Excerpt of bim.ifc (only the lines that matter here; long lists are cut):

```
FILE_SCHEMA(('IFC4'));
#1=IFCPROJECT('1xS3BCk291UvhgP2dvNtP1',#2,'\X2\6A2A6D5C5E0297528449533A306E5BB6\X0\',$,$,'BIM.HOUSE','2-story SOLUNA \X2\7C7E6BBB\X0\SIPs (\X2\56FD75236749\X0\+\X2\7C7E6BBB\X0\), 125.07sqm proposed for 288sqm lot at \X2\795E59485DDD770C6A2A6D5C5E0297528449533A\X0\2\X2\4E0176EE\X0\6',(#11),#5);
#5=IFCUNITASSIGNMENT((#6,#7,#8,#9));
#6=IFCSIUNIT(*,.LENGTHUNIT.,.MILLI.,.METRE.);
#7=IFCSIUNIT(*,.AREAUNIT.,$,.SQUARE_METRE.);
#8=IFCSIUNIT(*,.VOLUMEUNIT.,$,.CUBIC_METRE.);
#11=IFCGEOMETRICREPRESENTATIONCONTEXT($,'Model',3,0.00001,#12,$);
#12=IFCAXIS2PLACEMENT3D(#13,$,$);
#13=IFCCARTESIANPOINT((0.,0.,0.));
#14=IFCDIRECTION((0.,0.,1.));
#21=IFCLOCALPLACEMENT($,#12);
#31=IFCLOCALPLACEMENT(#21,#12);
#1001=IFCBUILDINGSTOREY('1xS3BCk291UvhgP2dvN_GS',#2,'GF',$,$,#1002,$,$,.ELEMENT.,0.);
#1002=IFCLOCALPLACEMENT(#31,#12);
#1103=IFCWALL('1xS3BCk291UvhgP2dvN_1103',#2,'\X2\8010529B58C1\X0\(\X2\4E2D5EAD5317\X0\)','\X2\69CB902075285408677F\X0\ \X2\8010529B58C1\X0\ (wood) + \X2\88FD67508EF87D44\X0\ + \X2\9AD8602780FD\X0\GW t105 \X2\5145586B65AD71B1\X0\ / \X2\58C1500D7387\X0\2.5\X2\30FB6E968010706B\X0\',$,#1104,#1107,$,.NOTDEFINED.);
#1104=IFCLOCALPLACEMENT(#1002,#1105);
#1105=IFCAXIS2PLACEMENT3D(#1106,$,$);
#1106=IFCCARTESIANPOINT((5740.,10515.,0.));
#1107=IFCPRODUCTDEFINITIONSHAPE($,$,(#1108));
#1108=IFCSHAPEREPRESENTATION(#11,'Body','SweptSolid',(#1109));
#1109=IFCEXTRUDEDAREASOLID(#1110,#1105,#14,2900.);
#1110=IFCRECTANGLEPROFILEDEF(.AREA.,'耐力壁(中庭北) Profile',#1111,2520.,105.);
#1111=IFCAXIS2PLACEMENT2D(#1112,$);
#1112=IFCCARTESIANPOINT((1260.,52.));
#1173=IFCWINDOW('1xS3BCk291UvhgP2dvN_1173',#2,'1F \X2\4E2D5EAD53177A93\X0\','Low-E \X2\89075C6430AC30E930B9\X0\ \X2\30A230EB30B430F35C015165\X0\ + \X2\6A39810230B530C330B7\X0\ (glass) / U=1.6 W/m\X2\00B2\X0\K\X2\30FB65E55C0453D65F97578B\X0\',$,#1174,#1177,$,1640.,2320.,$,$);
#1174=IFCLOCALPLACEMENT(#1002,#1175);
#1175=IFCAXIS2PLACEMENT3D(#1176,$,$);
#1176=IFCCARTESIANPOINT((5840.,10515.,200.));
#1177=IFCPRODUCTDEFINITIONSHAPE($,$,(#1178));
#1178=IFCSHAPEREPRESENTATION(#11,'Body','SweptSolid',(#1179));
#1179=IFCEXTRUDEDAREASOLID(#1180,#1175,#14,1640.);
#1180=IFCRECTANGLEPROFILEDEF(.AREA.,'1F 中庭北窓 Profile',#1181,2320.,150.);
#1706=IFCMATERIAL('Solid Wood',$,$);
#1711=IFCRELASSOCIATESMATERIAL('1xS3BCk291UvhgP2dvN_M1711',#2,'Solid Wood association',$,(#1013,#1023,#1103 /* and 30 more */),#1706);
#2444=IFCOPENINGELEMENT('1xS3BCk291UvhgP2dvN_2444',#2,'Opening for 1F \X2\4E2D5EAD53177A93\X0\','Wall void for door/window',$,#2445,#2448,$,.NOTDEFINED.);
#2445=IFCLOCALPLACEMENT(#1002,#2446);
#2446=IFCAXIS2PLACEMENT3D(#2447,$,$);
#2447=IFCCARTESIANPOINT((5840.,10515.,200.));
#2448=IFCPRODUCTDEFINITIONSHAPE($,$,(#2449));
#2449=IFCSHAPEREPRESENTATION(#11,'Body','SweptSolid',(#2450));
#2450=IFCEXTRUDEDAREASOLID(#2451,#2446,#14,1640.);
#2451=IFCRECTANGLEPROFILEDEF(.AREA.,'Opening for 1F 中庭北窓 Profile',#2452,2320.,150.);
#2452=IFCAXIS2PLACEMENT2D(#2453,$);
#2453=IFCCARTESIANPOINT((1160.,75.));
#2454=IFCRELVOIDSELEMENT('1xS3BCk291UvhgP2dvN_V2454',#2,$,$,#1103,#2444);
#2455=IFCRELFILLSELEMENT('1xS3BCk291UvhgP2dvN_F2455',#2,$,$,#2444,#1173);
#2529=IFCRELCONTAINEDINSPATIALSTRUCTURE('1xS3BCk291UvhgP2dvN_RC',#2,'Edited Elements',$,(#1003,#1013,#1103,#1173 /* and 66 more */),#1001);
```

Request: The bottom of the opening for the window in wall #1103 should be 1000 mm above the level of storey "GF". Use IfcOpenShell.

```python
import numpy as np
import ifcopenshell
import ifcopenshell.api.geometry
import ifcopenshell.geom
import ifcopenshell.util.element
import ifcopenshell.util.placement
import ifcopenshell.util.shape
import ifcopenshell.util.unit

model = ifcopenshell.open("bim.ifc")
unit_scale = ifcopenshell.util.unit.calculate_unit_scale(model)

window = model.by_guid("1xS3BCk291UvhgP2dvN_1173")
opening = window.FillsVoids[0].RelatingOpeningElement
storey = ifcopenshell.util.element.get_container(window, ifc_class="IfcBuildingStorey")
level = ifcopenshell.util.placement.get_local_placement(storey.ObjectPlacement)[2, 3]

# The opening's origin need not be at the sill, so measure its lowest point.
shape = ifcopenshell.geom.create_shape(ifcopenshell.geom.settings(), opening)
bottom = ifcopenshell.util.shape.get_shape_bottom_elevation(shape, shape.geometry) / unit_scale
dz = level + 1000.0 - bottom

shift = np.array([0.0, 0.0, dz])
# The window is not placed relative to its opening, so move both.
for product in (opening, window):
    matrix = ifcopenshell.util.placement.get_local_placement(product.ObjectPlacement)
    matrix[:3, 3] += shift
    ifcopenshell.api.geometry.edit_object_placement(model, product=product, matrix=matrix, is_si=False)

print(f"moved by {dz * unit_scale:+.3f} m")

model.write("bim_edited.ifc")
```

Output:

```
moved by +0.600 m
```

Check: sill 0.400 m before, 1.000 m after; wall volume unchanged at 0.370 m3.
